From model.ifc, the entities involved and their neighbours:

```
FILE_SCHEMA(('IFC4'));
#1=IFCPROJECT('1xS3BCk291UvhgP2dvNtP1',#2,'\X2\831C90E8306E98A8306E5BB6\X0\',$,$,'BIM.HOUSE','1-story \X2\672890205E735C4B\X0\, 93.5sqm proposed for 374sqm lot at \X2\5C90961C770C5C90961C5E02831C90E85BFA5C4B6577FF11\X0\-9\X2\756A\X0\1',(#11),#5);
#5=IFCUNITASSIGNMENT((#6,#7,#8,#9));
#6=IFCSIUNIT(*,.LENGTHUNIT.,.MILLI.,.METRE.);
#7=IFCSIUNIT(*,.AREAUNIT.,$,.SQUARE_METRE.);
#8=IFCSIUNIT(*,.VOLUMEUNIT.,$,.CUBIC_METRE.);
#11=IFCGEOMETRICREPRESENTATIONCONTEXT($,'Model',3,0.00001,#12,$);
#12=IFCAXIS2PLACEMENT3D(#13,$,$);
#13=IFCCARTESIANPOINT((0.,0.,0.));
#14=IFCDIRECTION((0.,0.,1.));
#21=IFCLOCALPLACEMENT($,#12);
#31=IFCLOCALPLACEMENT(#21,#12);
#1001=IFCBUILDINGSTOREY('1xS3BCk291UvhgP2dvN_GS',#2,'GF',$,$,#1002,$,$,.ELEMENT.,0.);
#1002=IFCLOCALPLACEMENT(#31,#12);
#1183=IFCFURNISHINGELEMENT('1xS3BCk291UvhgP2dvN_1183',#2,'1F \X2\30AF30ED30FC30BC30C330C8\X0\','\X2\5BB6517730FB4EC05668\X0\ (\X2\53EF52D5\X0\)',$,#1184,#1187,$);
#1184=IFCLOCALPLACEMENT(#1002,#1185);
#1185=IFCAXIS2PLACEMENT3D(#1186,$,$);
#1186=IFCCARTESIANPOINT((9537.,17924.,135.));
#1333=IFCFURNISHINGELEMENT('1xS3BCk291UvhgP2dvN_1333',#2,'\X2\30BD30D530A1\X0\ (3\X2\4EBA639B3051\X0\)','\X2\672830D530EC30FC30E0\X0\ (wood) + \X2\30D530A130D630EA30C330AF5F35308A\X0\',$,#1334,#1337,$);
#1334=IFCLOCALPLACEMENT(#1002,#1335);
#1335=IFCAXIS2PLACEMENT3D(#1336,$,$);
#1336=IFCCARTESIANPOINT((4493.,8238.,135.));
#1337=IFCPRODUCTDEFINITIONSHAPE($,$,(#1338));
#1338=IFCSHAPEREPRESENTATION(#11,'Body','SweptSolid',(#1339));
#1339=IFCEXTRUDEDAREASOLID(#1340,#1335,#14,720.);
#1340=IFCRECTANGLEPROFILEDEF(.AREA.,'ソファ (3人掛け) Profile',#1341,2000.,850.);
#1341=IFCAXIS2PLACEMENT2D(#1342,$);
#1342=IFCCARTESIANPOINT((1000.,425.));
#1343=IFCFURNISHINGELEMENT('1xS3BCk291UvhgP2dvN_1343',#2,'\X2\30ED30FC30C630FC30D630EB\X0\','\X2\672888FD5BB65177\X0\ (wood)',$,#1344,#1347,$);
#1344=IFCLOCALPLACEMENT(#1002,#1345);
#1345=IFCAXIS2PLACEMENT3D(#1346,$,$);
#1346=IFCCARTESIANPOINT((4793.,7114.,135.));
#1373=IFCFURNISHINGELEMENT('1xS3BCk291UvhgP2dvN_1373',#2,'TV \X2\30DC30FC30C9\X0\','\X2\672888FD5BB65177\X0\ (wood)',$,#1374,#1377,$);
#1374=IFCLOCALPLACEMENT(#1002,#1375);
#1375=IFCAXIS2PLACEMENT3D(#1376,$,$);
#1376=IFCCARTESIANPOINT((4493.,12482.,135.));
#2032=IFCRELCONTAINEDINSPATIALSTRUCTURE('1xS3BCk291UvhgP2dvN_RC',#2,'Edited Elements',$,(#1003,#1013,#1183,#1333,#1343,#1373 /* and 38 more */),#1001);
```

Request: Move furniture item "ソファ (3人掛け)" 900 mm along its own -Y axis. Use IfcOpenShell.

```python
import ifcopenshell
import ifcopenshell.api.geometry
import ifcopenshell.util.placement

model = ifcopenshell.open("model.ifc")

item = model.by_guid("1xS3BCk291UvhgP2dvN_1333")
matrix = ifcopenshell.util.placement.get_local_placement(item.ObjectPlacement)
matrix[:3, 3] -= matrix[:3, 1] * 900.0
ifcopenshell.api.geometry.edit_object_placement(model, product=item, matrix=matrix, is_si=False)

print(ifcopenshell.util.placement.get_local_placement(item.ObjectPlacement).round(3) + 0.0)

model.write("model_rev.ifc")
```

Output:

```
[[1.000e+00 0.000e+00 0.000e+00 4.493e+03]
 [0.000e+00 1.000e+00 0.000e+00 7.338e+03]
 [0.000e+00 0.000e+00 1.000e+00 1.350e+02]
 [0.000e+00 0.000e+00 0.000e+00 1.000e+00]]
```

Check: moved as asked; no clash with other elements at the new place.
